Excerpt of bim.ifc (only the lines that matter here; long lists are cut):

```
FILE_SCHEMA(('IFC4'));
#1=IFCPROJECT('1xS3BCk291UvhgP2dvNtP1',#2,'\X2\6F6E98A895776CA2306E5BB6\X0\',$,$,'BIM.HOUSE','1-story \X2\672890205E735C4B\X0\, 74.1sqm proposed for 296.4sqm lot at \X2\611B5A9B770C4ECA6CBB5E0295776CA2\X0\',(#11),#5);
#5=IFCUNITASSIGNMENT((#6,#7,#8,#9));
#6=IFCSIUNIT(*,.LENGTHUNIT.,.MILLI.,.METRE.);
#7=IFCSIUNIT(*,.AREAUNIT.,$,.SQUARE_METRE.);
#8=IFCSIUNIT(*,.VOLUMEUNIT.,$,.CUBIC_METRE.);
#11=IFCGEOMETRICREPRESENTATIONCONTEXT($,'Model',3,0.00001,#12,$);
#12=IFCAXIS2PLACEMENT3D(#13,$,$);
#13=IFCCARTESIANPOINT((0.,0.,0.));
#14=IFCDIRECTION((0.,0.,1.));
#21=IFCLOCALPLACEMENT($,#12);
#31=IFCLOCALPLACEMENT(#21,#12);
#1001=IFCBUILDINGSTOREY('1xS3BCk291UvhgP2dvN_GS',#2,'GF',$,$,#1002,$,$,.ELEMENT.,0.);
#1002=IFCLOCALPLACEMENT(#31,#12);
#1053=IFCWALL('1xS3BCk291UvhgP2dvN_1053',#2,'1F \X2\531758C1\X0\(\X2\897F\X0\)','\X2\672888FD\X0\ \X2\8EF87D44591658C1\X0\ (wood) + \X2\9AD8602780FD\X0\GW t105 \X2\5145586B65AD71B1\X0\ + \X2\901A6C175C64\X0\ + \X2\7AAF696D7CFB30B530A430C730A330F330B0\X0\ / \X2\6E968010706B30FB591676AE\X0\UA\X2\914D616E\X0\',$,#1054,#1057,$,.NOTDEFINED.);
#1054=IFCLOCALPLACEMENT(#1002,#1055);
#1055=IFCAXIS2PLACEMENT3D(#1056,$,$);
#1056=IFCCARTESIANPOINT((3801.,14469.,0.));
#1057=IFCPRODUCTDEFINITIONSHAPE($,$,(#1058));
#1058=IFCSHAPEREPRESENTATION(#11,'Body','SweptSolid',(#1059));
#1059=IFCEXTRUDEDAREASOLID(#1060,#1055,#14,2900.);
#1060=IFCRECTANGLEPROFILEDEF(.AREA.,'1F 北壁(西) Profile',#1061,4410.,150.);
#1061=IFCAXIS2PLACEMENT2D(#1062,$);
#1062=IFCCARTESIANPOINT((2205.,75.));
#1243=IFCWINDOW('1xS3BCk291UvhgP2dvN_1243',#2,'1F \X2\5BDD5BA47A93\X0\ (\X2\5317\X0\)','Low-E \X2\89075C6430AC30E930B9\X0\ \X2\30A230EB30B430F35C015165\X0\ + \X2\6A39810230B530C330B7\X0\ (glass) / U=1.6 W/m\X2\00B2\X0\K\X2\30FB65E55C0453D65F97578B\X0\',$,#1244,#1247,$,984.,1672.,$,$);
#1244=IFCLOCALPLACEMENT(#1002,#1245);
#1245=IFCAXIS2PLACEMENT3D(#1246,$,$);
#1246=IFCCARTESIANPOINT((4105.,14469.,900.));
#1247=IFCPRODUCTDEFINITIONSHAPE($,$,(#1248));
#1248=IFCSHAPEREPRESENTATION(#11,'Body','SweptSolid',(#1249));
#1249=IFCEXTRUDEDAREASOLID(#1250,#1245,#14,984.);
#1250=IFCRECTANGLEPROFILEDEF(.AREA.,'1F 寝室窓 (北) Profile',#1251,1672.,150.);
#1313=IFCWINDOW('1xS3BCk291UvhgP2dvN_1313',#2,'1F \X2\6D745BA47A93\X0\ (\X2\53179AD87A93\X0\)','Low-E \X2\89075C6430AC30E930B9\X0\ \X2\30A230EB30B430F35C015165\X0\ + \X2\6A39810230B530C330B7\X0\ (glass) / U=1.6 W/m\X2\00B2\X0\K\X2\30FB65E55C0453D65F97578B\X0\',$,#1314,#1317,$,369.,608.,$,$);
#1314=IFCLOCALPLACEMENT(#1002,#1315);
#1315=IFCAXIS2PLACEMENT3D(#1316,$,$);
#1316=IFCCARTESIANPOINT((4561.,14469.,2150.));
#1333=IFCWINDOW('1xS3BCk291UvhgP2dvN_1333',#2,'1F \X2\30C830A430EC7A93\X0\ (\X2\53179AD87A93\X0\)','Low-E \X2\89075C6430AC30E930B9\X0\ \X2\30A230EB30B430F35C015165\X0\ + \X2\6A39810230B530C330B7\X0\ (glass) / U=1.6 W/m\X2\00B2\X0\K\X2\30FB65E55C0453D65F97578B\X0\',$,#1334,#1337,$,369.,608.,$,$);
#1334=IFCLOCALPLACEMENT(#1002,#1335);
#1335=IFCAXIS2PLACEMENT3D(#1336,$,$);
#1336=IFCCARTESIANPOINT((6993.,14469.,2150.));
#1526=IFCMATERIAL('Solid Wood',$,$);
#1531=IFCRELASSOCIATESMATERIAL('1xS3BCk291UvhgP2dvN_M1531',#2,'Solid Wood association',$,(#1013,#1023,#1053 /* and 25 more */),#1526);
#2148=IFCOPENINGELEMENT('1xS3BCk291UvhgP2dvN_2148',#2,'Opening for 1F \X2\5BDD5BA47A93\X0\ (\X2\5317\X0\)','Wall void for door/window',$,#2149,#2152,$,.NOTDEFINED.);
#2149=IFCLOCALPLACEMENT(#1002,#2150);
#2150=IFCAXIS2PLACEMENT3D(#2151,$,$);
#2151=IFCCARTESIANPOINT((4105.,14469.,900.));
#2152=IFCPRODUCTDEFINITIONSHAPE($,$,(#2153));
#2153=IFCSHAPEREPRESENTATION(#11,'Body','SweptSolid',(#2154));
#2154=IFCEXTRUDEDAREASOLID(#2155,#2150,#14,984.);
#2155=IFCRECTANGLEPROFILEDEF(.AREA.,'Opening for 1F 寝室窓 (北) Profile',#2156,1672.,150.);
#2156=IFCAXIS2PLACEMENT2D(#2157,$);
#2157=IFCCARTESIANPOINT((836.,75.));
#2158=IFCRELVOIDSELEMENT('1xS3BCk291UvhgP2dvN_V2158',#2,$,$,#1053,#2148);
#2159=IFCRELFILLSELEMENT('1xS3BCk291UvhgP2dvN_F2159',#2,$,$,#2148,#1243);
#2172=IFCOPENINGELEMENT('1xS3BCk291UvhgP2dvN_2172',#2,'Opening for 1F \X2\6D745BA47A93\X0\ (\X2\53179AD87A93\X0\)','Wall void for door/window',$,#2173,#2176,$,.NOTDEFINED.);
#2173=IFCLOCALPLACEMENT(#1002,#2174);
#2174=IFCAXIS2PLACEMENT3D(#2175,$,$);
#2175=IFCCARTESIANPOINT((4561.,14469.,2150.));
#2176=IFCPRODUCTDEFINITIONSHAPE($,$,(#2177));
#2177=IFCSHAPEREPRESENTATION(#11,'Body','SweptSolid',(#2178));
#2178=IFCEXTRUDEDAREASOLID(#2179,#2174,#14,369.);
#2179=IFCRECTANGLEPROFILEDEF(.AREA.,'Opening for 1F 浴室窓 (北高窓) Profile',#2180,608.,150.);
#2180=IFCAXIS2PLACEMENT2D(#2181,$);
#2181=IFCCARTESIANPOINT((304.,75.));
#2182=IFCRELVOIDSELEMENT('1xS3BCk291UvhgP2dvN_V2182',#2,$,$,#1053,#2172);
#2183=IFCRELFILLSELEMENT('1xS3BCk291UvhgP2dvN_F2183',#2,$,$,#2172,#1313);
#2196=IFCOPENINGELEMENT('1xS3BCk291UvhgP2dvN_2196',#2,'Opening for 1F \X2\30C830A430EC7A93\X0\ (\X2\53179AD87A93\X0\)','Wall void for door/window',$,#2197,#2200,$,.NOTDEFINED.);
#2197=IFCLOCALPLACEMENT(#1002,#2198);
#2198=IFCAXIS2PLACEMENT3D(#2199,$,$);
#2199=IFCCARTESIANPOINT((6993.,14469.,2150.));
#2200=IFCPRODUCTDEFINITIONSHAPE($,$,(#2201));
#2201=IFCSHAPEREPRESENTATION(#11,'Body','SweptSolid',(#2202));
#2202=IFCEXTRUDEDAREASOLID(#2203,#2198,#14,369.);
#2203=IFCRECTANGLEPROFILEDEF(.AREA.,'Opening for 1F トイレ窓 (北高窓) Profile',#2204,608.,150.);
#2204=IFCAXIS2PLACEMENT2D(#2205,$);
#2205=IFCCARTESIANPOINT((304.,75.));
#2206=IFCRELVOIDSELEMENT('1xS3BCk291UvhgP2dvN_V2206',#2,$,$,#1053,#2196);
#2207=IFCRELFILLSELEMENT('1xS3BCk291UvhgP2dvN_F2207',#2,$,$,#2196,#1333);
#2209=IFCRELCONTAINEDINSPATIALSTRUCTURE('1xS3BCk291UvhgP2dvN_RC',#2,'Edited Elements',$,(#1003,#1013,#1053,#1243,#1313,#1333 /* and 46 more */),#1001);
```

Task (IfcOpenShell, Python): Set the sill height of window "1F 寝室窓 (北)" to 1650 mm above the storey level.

```python
import numpy as np
import ifcopenshell
import ifcopenshell.api.geometry
import ifcopenshell.geom
import ifcopenshell.util.element
import ifcopenshell.util.placement
import ifcopenshell.util.shape
import ifcopenshell.util.unit

model = ifcopenshell.open("bim.ifc")
unit_scale = ifcopenshell.util.unit.calculate_unit_scale(model)

window = model.by_id(1243)
opening = window.FillsVoids[0].RelatingOpeningElement
storey = ifcopenshell.util.element.get_container(window, ifc_class="IfcBuildingStorey")
level = ifcopenshell.util.placement.get_local_placement(storey.ObjectPlacement)[2, 3]

# The opening's origin need not be at the sill, so measure its lowest point.
shape = ifcopenshell.geom.create_shape(ifcopenshell.geom.settings(), opening)
bottom = ifcopenshell.util.shape.get_shape_bottom_elevation(shape, shape.geometry) / unit_scale
dz = level + 1.65 / unit_scale - bottom

shift = np.array([0.0, 0.0, dz])
# The window is not placed relative to its opening, so move both.
for product in (opening, window):
    matrix = ifcopenshell.util.placement.get_local_placement(product.ObjectPlacement)
    matrix[:3, 3] += shift
    ifcopenshell.api.geometry.edit_object_placement(model, product=product, matrix=matrix, is_si=False)

print(f"moved by {dz * unit_scale:+.3f} m")

model.write("bim_v2.ifc")
```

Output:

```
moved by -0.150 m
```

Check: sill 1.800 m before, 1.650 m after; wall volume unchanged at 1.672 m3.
